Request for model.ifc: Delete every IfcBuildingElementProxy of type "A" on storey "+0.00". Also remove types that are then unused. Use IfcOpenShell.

First a look at what the model holds.

```python
import ifcopenshell
import ifcopenshell.util.element

model = ifcopenshell.open("model.ifc")
print(model.schema)
storey = next(s for s in model.by_type("IfcBuildingStorey") if s.Name == "+0.00")
proxies = [e for e in ifcopenshell.util.element.get_decomposition(storey) if e.is_a("IfcBuildingElementProxy")]
seen = {}
for e in proxies:
    element_type = ifcopenshell.util.element.get_type(e)
    name = element_type.Name if element_type not in (None, e) else None
    seen[name] = seen.get(name, 0) + 1
for name, count in sorted(seen.items(), key=str):
    print(count, "x", name)
```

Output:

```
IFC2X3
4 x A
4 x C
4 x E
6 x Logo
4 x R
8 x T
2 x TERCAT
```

```python
import ifcopenshell
import ifcopenshell.api.root
import ifcopenshell.util.element

model = ifcopenshell.open("model.ifc")

storey = next(s for s in model.by_type("IfcBuildingStorey") if s.Name == "+0.00")
proxies = [e for e in ifcopenshell.util.element.get_decomposition(storey) if e.is_a("IfcBuildingElementProxy")]
targets = [e for e in proxies if (t := ifcopenshell.util.element.get_type(e)) not in (None, e) and t.Name == "A"]
types = {ifcopenshell.util.element.get_type(e) for e in targets} - {None, *targets}

for e in targets:
    ifcopenshell.api.root.remove_product(model, product=e)
print(len(targets), "removed")

unused = [t for t in types if not ifcopenshell.util.element.get_types(t)]
for t in unused:
    ifcopenshell.api.root.remove_product(model, product=t)
print(len(unused), "unused types removed")

model.write("model_rev.ifc")
```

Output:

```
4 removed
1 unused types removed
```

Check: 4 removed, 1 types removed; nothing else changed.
